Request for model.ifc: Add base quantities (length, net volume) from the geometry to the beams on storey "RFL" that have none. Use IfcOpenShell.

First a look at what the model holds.

```python
import ifcopenshell
import ifcopenshell.util.element
import ifcopenshell.util.unit

model = ifcopenshell.open("model.ifc")
print(model.schema)
for unit_type in ("LENGTHUNIT", "AREAUNIT", "VOLUMEUNIT"):
    print(unit_type, ifcopenshell.util.unit.calculate_unit_scale(model, unit_type))
storey = next(s for s in model.by_type("IfcBuildingStorey") if s.Name == "RFL")
beams = [e for e in ifcopenshell.util.element.get_decomposition(storey) if e.is_a("IfcBeam")]
for e in sorted(beams, key=lambda e: e.id()):
    print(e.id(), e.is_a(), e.Name, list(ifcopenshell.util.element.get_psets(e, qtos_only=True)), sep=" | ")
```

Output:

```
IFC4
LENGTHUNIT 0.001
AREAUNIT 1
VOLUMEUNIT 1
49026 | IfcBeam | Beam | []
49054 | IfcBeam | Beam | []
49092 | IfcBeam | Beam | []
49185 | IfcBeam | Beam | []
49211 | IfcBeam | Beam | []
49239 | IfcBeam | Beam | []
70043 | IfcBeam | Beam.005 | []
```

```python
import ifcopenshell
import ifcopenshell.api.pset
import ifcopenshell.geom
import ifcopenshell.util.element
import ifcopenshell.util.shape
import ifcopenshell.util.unit

model = ifcopenshell.open("model.ifc")
unit_scale = ifcopenshell.util.unit.calculate_unit_scale(model)
volume_scale = ifcopenshell.util.unit.calculate_unit_scale(model, "VOLUMEUNIT")
settings = ifcopenshell.geom.settings()

storey = next(s for s in model.by_type("IfcBuildingStorey") if s.Name == "RFL")
beams = [e for e in ifcopenshell.util.element.get_decomposition(storey) if e.is_a("IfcBeam")]

for e in sorted(beams, key=lambda e: e.id()):
    if ifcopenshell.util.element.get_psets(e, qtos_only=True, should_inherit=False):
        continue
    # Geometry comes back in metres, in the element's own axes.
    shape = ifcopenshell.geom.create_shape(settings, e)
    values = {
        "Length": ifcopenshell.util.shape.get_max_xyz(shape.geometry) / unit_scale,
        "NetVolume": ifcopenshell.util.shape.get_volume(shape.geometry) / volume_scale,
    }
    qto = ifcopenshell.api.pset.add_qto(model, product=e, name="Qto_BeamBaseQuantities")
    ifcopenshell.api.pset.edit_qto(model, qto=qto, properties=values)
    print(e.id(), {k: round(v, 3) for k, v in values.items()})

model.write("model-out.ifc")
```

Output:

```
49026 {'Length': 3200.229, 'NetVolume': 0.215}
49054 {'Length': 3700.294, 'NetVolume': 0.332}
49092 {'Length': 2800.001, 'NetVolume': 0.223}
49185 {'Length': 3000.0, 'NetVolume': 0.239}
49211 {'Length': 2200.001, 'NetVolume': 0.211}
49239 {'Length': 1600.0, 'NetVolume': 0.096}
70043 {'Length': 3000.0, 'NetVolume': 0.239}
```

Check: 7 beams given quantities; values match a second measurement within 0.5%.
